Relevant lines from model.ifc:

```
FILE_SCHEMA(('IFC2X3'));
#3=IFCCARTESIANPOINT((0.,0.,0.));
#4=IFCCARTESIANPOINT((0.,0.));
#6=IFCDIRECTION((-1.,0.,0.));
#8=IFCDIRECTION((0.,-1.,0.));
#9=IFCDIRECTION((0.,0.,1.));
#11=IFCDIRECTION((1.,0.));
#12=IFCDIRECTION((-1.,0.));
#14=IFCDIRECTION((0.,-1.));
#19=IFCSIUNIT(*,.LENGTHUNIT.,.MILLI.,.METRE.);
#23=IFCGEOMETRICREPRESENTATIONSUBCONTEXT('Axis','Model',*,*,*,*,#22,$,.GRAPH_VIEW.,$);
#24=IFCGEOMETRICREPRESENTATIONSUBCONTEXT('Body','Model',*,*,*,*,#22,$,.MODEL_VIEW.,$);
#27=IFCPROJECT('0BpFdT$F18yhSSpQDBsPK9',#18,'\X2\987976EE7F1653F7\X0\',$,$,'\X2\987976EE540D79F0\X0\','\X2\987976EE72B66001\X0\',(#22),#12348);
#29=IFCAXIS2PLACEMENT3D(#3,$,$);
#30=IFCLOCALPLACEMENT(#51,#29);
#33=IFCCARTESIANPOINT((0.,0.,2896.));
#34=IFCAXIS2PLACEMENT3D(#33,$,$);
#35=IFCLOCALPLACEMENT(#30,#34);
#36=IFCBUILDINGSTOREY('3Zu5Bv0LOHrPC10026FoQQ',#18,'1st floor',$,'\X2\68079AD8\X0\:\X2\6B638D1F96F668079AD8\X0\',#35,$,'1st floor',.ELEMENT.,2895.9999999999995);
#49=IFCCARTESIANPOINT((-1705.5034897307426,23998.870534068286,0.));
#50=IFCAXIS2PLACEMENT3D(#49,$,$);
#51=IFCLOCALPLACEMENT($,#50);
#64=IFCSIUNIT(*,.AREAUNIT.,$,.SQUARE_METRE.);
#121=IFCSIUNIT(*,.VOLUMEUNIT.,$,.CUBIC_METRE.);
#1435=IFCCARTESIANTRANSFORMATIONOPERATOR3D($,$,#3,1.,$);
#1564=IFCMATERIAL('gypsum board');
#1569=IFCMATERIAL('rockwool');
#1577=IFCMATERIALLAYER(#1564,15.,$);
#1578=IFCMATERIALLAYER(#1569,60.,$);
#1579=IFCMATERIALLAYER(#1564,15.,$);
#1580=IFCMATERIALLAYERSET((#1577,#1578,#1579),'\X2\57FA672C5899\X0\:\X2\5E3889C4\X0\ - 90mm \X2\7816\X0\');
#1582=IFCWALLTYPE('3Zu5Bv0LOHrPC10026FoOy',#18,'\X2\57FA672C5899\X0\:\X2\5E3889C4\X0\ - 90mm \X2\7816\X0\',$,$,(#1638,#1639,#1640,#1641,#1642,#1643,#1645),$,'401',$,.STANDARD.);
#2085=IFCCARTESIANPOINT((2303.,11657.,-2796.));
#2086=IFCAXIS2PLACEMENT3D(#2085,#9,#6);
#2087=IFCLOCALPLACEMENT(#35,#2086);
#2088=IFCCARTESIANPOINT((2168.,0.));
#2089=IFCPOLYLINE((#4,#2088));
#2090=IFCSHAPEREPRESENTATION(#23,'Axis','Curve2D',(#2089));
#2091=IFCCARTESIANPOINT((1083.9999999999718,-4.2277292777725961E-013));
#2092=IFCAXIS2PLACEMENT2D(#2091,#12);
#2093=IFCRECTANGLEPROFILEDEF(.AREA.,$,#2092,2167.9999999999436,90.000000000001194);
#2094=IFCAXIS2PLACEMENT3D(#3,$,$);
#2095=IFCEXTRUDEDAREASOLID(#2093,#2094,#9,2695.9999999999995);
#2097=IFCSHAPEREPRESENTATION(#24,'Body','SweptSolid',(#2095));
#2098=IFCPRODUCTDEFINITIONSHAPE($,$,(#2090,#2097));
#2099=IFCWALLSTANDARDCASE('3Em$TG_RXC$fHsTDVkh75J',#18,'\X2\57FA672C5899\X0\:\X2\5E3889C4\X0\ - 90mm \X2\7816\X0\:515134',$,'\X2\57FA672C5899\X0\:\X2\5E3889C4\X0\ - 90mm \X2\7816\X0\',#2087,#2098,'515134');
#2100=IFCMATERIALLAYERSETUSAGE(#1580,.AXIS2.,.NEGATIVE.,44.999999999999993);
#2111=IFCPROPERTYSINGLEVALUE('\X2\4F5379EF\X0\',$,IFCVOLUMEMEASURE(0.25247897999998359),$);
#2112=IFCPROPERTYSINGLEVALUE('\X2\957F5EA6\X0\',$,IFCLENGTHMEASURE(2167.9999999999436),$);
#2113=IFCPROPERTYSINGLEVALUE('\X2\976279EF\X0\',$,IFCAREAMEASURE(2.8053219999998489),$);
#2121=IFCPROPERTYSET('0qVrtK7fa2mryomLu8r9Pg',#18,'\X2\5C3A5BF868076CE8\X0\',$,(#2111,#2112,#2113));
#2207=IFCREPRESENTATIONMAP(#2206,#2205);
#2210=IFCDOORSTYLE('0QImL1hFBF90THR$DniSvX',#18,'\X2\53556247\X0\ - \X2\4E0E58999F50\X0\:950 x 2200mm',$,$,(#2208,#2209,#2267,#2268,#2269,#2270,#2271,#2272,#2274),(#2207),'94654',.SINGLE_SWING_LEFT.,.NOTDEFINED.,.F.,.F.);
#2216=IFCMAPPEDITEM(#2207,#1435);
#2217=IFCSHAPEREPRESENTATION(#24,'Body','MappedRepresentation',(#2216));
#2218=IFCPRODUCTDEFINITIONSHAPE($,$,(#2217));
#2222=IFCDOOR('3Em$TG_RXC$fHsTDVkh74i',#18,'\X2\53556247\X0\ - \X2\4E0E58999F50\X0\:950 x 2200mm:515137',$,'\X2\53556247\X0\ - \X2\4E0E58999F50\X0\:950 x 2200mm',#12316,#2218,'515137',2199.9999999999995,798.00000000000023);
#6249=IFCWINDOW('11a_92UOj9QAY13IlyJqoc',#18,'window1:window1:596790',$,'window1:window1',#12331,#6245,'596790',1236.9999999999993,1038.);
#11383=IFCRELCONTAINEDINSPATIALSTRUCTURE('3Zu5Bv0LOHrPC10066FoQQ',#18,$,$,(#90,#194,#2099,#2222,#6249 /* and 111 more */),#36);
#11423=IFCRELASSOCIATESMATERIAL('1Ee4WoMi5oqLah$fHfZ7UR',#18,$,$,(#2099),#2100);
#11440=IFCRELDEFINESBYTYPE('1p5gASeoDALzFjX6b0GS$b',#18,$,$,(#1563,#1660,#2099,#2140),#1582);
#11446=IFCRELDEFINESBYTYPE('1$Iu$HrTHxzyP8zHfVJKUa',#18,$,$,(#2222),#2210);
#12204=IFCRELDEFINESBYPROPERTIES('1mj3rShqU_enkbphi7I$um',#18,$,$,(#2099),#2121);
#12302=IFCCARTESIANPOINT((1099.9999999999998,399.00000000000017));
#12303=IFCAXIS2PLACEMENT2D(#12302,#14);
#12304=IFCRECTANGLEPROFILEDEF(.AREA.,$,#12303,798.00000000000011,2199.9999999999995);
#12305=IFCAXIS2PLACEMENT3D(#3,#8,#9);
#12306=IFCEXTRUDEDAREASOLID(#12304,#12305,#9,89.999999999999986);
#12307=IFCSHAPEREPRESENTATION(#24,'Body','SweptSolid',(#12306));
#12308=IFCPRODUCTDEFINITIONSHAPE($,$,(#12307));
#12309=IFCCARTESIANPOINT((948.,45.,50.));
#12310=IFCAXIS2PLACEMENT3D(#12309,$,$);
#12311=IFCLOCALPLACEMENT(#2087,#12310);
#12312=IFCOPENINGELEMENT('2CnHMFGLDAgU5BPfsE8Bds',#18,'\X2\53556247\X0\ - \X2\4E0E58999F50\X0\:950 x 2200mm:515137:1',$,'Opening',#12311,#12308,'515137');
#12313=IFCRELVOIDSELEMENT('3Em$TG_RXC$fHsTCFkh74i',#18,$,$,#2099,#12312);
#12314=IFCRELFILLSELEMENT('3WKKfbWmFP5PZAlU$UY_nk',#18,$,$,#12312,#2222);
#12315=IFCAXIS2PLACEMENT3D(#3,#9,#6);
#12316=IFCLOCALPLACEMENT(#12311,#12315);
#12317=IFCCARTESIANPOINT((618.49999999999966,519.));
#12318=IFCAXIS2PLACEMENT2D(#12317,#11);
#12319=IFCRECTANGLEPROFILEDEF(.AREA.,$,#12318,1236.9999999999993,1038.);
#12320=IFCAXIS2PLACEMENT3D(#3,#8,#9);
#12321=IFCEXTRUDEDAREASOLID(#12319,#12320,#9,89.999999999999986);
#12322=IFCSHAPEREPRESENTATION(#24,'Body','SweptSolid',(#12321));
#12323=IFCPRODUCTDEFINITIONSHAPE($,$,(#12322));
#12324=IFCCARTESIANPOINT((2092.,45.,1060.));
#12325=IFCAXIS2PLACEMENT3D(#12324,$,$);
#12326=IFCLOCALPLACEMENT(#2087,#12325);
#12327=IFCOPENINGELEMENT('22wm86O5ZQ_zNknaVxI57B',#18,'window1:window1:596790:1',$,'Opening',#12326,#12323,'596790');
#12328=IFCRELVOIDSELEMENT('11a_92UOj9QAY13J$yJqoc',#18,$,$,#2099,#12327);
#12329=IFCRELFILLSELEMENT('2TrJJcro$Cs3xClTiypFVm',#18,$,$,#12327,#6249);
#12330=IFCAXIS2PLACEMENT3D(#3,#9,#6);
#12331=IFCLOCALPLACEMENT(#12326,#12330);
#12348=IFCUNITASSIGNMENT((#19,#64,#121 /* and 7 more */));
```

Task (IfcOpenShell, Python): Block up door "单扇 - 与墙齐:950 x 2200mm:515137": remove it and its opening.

```python
import ifcopenshell
import ifcopenshell.api.feature
import ifcopenshell.api.pset
import ifcopenshell.api.root
import ifcopenshell.geom
import ifcopenshell.util.element
import ifcopenshell.util.shape
import ifcopenshell.util.unit

model = ifcopenshell.open("model.ifc")
area_scale = ifcopenshell.util.unit.calculate_unit_scale(model, "AREAUNIT")
volume_scale = ifcopenshell.util.unit.calculate_unit_scale(model, "VOLUMEUNIT")
settings = ifcopenshell.geom.settings()


def volume(element):
    """Net volume in cubic metres, openings subtracted."""
    shape = ifcopenshell.geom.create_shape(settings, element)
    return ifcopenshell.util.shape.get_volume(shape.geometry)


door = model.by_id(2222)
opening = door.FillsVoids[0].RelatingOpeningElement
wall = opening.VoidsElements[0].RelatingBuildingElement
before = volume(wall)

ifcopenshell.api.root.remove_product(model, product=door)
ifcopenshell.api.feature.remove_feature(model, feature=opening)

after = volume(wall)
thickness = 0.09  # wall thickness in metres

# Update the wall's stored quantities.
pset = model.by_id(ifcopenshell.util.element.get_pset(wall, "尺寸标注", should_inherit=False)["id"])
ifcopenshell.api.pset.edit_pset(model, pset=pset, properties={
    "体积": model.create_entity("IfcVolumeMeasure", after / volume_scale),
    "面积": model.create_entity("IfcAreaMeasure", after / thickness / area_scale),
})

print(f"wall volume {before:.3f} -> {after:.3f} m3")

model.write("model_rev.ifc")
```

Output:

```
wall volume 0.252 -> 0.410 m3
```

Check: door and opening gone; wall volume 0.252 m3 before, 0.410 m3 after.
